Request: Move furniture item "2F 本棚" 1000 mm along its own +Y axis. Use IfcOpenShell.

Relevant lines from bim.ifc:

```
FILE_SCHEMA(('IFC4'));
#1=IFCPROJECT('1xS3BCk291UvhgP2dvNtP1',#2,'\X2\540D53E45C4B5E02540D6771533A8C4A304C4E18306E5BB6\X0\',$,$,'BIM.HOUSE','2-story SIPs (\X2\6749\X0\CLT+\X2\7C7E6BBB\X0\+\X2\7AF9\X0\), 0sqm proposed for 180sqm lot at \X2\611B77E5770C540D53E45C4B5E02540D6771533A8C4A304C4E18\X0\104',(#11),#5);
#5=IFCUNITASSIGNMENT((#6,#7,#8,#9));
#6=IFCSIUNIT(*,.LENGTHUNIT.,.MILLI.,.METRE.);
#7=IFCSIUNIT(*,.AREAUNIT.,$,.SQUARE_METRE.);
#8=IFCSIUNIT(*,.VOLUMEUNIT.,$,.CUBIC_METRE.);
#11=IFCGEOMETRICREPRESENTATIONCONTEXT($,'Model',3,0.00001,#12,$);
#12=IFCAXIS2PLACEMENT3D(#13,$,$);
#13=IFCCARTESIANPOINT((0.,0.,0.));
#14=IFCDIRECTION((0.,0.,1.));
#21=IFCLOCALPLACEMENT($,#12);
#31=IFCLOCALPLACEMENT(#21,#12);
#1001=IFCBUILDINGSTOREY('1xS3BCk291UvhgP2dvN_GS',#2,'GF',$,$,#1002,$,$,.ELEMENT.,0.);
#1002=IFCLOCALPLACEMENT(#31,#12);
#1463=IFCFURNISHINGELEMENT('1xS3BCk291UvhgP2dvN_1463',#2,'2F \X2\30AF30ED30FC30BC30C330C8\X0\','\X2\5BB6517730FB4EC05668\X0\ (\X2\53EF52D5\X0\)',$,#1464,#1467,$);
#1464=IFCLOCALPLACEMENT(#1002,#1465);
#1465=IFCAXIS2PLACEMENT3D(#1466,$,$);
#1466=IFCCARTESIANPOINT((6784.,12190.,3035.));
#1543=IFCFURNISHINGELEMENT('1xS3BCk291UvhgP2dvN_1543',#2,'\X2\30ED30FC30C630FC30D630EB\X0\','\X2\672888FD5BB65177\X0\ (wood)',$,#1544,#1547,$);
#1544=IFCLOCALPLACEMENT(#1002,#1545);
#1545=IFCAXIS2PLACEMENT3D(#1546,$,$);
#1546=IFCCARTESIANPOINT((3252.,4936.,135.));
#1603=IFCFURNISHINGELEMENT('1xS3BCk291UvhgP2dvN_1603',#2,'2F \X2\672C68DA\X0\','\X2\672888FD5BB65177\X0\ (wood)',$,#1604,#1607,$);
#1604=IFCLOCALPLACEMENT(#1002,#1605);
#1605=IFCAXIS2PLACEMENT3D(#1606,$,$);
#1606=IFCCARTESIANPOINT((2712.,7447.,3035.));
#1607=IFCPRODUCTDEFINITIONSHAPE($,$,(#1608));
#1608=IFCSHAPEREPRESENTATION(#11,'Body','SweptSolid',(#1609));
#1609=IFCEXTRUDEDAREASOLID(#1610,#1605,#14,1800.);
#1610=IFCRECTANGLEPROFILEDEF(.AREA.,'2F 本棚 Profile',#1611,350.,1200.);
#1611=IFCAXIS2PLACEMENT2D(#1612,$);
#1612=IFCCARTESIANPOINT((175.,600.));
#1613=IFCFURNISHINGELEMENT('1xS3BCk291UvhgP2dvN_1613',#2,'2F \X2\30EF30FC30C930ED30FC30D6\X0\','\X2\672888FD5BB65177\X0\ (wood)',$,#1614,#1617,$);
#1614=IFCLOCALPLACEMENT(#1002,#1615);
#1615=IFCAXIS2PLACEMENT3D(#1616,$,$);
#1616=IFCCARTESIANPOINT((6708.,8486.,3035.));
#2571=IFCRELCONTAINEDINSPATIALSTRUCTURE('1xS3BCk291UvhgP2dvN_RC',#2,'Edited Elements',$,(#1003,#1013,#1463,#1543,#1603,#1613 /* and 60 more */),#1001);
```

```python
import ifcopenshell
import ifcopenshell.api.geometry
import ifcopenshell.util.placement
import ifcopenshell.util.unit

model = ifcopenshell.open("bim.ifc")
unit_scale = ifcopenshell.util.unit.calculate_unit_scale(model)

item = model.by_guid("1xS3BCk291UvhgP2dvN_1603")
matrix = ifcopenshell.util.placement.get_local_placement(item.ObjectPlacement)
matrix[:3, 3] += matrix[:3, 1] * 1 / unit_scale
ifcopenshell.api.geometry.edit_object_placement(model, product=item, matrix=matrix, is_si=False)

print(ifcopenshell.util.placement.get_local_placement(item.ObjectPlacement).round(3) + 0.0)

model.write("bim_rev.ifc")
```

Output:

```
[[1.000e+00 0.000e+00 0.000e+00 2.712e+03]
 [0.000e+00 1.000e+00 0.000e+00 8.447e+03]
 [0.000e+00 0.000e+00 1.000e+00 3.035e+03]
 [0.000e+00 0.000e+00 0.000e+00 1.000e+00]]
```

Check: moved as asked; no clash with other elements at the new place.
